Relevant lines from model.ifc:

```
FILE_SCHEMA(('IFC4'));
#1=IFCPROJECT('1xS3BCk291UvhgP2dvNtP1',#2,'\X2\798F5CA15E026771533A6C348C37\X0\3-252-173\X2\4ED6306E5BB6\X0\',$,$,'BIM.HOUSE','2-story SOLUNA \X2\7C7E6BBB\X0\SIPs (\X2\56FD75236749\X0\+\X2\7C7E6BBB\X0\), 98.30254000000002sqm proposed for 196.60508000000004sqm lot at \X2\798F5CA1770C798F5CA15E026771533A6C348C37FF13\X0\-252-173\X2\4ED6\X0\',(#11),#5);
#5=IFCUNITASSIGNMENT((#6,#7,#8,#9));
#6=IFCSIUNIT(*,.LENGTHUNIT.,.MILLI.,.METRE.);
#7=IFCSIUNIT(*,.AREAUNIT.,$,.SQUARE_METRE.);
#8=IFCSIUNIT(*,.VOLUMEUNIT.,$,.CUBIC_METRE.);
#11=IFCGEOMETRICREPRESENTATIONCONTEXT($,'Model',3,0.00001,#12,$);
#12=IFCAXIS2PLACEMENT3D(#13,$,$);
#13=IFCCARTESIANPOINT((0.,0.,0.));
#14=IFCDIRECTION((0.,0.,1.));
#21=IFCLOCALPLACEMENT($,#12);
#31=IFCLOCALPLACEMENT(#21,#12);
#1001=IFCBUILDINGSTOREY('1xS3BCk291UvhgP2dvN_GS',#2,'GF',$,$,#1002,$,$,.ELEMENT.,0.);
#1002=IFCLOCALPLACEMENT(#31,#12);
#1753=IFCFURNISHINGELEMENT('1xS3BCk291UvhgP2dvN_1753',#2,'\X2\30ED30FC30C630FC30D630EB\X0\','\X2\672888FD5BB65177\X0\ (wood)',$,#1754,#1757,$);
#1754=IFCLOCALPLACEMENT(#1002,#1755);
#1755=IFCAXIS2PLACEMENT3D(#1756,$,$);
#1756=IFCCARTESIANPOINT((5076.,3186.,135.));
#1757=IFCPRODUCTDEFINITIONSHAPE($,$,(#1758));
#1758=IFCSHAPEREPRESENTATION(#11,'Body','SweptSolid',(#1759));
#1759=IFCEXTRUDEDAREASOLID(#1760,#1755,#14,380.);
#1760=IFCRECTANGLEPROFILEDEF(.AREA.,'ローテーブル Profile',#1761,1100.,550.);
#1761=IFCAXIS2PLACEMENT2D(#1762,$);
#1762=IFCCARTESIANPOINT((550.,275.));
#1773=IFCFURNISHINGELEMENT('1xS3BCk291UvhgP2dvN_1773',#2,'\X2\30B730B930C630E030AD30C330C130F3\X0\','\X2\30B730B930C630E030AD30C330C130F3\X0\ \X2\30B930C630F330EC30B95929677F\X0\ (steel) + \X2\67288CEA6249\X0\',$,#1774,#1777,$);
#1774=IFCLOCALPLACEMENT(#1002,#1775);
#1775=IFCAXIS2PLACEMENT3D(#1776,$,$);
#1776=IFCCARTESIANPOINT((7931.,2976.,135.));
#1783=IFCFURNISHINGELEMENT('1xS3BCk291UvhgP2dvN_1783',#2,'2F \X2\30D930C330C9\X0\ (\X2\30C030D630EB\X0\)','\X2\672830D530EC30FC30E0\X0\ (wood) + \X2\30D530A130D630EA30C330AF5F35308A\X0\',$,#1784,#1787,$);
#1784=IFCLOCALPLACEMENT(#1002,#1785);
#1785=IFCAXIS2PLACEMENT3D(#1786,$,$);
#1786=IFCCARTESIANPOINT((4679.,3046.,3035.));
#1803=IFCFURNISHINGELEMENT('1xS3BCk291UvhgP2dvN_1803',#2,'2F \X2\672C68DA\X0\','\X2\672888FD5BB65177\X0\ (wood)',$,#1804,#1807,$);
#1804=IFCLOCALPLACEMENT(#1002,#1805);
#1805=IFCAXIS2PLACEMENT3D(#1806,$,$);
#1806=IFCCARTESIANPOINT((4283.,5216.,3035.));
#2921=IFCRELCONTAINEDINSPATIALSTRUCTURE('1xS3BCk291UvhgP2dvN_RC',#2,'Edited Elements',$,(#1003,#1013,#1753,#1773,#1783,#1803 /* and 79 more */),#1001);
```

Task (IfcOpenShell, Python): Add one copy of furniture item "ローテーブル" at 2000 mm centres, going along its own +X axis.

```python
import ifcopenshell
import ifcopenshell.api.geometry
import ifcopenshell.api.root
import ifcopenshell.util.element
import ifcopenshell.util.placement
import ifcopenshell.util.unit

model = ifcopenshell.open("model.ifc")
unit_scale = ifcopenshell.util.unit.calculate_unit_scale(model)


def reuse_history(source, copy):
    """copy_class also copies each property set's owner history, people and application; keep the originals."""
    for rel in copy.IsDefinedBy:
        if rel.is_a("IfcRelDefinesByProperties") and (history := rel.RelatingPropertyDefinition.OwnerHistory):
            rel.RelatingPropertyDefinition.OwnerHistory = source.OwnerHistory
            ifcopenshell.util.element.remove_deep2(model, history)


source = model.by_id(1753)
base = ifcopenshell.util.placement.get_local_placement(source.ObjectPlacement)
step = base[:3, 0] * 2 / unit_scale

for i in range(1, 2):
    copy = ifcopenshell.api.root.copy_class(model, product=source)
    copy.Representation = ifcopenshell.util.element.copy_deep(
        model, source.Representation, exclude=["IfcGeometricRepresentationContext", "IfcRepresentationMap"]
    )
    reuse_history(source, copy)
    matrix = base.copy()
    matrix[:3, 3] += i * step
    print("added at", matrix[:3, 3].round(3) + 0.0)
    ifcopenshell.api.geometry.edit_object_placement(model, product=copy, matrix=matrix, is_si=False)

model.write("model_updated.ifc")
```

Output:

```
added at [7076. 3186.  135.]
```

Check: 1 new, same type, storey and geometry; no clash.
